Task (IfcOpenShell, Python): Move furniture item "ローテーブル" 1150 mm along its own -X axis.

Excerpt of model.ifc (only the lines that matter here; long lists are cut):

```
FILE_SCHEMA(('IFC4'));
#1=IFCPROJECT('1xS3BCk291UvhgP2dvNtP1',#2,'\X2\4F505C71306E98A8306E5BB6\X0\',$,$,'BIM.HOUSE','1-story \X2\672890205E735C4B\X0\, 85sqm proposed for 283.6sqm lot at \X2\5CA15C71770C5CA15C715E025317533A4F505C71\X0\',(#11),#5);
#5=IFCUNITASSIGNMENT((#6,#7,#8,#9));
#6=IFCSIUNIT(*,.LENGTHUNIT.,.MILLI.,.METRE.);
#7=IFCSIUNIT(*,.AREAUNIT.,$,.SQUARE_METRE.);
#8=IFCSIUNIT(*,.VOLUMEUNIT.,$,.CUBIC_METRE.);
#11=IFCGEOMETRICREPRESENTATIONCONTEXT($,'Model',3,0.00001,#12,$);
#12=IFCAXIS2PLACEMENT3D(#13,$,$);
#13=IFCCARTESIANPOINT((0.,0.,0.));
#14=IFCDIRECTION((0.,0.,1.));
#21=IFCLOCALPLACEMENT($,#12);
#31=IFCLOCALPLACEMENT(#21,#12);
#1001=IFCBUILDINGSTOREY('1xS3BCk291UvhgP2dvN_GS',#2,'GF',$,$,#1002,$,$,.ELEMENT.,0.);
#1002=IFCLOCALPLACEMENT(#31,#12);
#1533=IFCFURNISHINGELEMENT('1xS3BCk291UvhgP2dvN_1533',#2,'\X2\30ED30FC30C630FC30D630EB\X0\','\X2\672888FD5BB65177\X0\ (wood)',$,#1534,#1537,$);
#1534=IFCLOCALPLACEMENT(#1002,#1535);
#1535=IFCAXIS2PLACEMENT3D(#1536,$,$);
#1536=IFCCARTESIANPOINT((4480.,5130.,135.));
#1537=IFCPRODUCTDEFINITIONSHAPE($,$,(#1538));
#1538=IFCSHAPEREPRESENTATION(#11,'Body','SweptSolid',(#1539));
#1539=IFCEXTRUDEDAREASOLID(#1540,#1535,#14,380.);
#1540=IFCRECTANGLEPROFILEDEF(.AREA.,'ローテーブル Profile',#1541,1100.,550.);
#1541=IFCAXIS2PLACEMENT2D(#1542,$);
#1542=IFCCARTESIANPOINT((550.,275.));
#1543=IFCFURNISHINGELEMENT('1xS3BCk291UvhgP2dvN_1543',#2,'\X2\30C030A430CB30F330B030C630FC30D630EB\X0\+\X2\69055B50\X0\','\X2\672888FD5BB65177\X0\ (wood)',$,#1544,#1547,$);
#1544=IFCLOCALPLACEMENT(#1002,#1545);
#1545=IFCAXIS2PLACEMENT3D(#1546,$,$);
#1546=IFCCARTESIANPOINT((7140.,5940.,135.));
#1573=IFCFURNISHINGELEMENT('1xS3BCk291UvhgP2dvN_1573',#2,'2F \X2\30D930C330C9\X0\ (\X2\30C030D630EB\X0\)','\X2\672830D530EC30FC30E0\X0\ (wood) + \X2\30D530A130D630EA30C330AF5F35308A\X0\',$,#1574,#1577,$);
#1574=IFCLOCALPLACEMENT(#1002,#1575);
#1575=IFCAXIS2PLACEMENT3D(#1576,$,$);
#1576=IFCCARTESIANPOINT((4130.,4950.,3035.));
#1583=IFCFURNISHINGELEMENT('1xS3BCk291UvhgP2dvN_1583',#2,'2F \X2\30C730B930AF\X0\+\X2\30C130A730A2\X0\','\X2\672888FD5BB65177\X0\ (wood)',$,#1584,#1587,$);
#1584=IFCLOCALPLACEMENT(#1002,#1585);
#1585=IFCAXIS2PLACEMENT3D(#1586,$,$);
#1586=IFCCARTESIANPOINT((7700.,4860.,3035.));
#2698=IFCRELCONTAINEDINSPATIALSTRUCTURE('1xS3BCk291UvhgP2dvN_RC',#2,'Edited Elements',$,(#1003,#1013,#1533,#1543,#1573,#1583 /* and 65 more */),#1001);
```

```python
import ifcopenshell
import ifcopenshell.api.geometry
import ifcopenshell.util.placement

model = ifcopenshell.open("model.ifc")

item = model.by_guid("1xS3BCk291UvhgP2dvN_1533")
matrix = ifcopenshell.util.placement.get_local_placement(item.ObjectPlacement)
matrix[:3, 3] -= matrix[:3, 0] * 1150.0
ifcopenshell.api.geometry.edit_object_placement(model, product=item, matrix=matrix, is_si=False)

print(ifcopenshell.util.placement.get_local_placement(item.ObjectPlacement).round(3) + 0.0)

model.write("model-out.ifc")
```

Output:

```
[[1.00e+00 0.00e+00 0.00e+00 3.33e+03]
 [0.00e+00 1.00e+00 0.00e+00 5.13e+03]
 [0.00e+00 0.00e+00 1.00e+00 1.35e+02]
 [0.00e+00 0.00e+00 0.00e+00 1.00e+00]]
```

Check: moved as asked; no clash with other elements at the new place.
